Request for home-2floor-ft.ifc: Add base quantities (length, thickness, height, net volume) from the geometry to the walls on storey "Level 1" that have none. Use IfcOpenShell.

First a look at what the model holds.

```python
import ifcopenshell
import ifcopenshell.util.element
import ifcopenshell.util.unit

model = ifcopenshell.open("home-2floor-ft.ifc")
print(model.schema)
for unit_type in ("LENGTHUNIT", "AREAUNIT", "VOLUMEUNIT"):
    print(unit_type, ifcopenshell.util.unit.calculate_unit_scale(model, unit_type))
storey = next(s for s in model.by_type("IfcBuildingStorey") if s.Name == "Level 1")
walls = [e for e in ifcopenshell.util.element.get_decomposition(storey) if e.is_a("IfcWall")]
for e in sorted(walls, key=lambda e: e.id()):
    print(e.id(), e.is_a(), e.Name, list(ifcopenshell.util.element.get_psets(e, qtos_only=True)), sep=" | ")
```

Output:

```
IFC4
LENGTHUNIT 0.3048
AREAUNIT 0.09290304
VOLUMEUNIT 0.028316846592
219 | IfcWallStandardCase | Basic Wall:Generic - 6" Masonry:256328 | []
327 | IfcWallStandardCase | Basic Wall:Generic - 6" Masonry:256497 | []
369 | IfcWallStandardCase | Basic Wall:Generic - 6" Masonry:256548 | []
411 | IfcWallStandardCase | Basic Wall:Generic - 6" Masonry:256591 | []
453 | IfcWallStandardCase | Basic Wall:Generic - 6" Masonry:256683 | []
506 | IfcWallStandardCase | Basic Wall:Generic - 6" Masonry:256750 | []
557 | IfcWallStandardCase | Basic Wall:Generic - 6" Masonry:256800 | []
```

```python
import ifcopenshell
import ifcopenshell.api.pset
import ifcopenshell.geom
import ifcopenshell.util.element
import ifcopenshell.util.shape
import ifcopenshell.util.unit

model = ifcopenshell.open("home-2floor-ft.ifc")
unit_scale = ifcopenshell.util.unit.calculate_unit_scale(model)
volume_scale = ifcopenshell.util.unit.calculate_unit_scale(model, "VOLUMEUNIT")
settings = ifcopenshell.geom.settings()

storey = next(s for s in model.by_type("IfcBuildingStorey") if s.Name == "Level 1")
walls = [e for e in ifcopenshell.util.element.get_decomposition(storey) if e.is_a("IfcWall")]

for e in sorted(walls, key=lambda e: e.id()):
    if ifcopenshell.util.element.get_psets(e, qtos_only=True, should_inherit=False):
        continue
    # Geometry comes back in metres, in the element's own axes.
    shape = ifcopenshell.geom.create_shape(settings, e)
    values = {
        "Length": ifcopenshell.util.shape.get_x(shape.geometry) / unit_scale,
        "Width": ifcopenshell.util.shape.get_y(shape.geometry) / unit_scale,
        "Height": ifcopenshell.util.shape.get_z(shape.geometry) / unit_scale,
        "NetVolume": ifcopenshell.util.shape.get_volume(shape.geometry) / volume_scale,
    }
    qto = ifcopenshell.api.pset.add_qto(model, product=e, name="Qto_WallBaseQuantities")
    ifcopenshell.api.pset.edit_qto(model, qto=qto, properties=values)
    print(e.id(), {k: round(v, 3) for k, v in values.items()})

model.write("home-2floor-ft-out.ifc")
```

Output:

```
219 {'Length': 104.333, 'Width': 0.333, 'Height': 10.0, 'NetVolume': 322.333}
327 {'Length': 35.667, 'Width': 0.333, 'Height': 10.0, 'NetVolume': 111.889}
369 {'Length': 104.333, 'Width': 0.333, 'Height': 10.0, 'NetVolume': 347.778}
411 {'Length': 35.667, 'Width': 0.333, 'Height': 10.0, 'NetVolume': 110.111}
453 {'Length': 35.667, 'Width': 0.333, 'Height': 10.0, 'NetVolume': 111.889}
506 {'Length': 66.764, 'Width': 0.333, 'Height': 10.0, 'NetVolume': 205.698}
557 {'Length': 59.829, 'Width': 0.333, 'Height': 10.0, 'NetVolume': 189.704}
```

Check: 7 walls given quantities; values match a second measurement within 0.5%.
